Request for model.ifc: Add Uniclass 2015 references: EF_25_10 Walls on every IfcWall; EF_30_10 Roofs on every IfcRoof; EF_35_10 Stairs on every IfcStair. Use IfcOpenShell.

First a look at what the model holds.

```python
import ifcopenshell

model = ifcopenshell.open("model.ifc")
print(model.schema)
print("classifications:", [c.Name for c in model.by_type("IfcClassification")])
for ifc_class in ("IfcDoor", "IfcRoof", "IfcStair", "IfcWall", "IfcWindow"):
    print(ifc_class, len(model.by_type(ifc_class)))
```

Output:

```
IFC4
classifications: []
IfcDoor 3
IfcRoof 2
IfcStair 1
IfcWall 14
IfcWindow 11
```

```python
import ifcopenshell
import ifcopenshell.api.classification

model = ifcopenshell.open("model.ifc")

system = ifcopenshell.api.classification.add_classification(model, classification="Uniclass 2015")

codes = {
    "IfcWall": ("EF_25_10", "Walls"),
    "IfcRoof": ("EF_30_10", "Roofs"),
    "IfcStair": ("EF_35_10", "Stairs"),
}
for ifc_class, (code, name) in codes.items():
    products = model.by_type(ifc_class)
    ifcopenshell.api.classification.add_reference(
        model, products=products, classification=system, identification=code, name=name
    )
    print(code, len(products))

model.write("model_rev.ifc")
```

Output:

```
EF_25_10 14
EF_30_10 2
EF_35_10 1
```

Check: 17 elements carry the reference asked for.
